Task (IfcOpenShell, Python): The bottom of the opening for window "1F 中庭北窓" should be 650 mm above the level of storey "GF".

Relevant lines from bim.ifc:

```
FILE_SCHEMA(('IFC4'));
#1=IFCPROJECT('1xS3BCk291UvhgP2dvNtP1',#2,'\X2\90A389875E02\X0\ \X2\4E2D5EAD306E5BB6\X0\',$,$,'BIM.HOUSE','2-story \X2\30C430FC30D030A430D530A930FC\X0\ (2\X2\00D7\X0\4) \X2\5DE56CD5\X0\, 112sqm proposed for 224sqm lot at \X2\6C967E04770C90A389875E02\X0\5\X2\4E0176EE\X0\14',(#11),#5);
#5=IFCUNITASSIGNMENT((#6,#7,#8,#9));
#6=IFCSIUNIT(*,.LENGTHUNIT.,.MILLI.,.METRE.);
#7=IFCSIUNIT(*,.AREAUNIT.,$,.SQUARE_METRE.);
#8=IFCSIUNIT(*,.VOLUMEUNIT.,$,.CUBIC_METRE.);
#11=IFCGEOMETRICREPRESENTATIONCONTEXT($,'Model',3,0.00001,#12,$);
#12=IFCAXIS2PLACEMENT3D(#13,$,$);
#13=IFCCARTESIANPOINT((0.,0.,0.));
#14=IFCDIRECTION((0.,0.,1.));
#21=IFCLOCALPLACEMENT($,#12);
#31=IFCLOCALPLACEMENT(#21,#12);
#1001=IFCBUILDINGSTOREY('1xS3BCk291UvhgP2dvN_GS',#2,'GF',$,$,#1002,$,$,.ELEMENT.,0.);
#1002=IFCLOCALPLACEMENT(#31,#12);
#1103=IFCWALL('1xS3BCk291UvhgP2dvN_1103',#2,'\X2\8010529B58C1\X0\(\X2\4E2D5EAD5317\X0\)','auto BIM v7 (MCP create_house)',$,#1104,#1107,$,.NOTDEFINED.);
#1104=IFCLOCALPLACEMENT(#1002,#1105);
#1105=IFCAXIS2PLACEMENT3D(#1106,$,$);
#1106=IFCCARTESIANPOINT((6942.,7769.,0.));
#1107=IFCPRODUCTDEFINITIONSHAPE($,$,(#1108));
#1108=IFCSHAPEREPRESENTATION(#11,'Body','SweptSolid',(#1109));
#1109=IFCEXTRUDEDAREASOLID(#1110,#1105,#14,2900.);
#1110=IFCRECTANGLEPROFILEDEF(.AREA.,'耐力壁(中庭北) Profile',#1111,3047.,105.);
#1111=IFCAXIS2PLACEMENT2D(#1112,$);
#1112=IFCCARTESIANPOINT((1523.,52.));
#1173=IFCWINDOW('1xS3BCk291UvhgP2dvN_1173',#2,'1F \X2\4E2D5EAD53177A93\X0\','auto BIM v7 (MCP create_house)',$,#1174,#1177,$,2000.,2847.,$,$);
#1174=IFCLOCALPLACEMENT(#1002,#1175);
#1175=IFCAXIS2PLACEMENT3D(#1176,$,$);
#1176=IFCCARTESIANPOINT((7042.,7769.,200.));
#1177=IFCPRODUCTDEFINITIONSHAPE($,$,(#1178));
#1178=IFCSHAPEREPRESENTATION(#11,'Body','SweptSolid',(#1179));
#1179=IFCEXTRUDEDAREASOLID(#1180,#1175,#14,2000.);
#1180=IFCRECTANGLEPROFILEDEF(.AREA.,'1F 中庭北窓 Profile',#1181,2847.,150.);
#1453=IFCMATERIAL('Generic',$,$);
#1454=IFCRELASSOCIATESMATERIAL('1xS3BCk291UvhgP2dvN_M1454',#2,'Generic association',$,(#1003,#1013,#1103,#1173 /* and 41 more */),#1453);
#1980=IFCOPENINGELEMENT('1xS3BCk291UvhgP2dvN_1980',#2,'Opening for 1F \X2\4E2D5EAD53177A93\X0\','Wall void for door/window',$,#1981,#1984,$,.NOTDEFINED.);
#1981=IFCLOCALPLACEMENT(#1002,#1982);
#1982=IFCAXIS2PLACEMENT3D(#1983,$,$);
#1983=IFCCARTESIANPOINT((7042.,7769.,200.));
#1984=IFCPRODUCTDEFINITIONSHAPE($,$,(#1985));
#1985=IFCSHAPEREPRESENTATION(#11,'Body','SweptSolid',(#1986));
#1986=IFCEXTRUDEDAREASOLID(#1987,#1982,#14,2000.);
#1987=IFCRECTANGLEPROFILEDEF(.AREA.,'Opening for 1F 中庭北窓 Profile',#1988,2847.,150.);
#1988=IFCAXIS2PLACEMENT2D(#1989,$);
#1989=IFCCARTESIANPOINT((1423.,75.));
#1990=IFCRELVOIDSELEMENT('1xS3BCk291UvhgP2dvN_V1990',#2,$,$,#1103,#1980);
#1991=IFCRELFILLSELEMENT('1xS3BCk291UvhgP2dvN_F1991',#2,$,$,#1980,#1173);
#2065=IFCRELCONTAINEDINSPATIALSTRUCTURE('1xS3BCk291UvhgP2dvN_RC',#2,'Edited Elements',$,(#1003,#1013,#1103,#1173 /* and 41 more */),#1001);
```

```python
import numpy as np
import ifcopenshell
import ifcopenshell.api.geometry
import ifcopenshell.geom
import ifcopenshell.util.element
import ifcopenshell.util.placement
import ifcopenshell.util.shape
import ifcopenshell.util.unit

model = ifcopenshell.open("bim.ifc")
unit_scale = ifcopenshell.util.unit.calculate_unit_scale(model)

window = model.by_guid("1xS3BCk291UvhgP2dvN_1173")
opening = window.FillsVoids[0].RelatingOpeningElement
storey = ifcopenshell.util.element.get_container(window, ifc_class="IfcBuildingStorey")
level = ifcopenshell.util.placement.get_local_placement(storey.ObjectPlacement)[2, 3]

# The opening's origin need not be at the sill, so measure its lowest point.
shape = ifcopenshell.geom.create_shape(ifcopenshell.geom.settings(), opening)
bottom = ifcopenshell.util.shape.get_shape_bottom_elevation(shape, shape.geometry) / unit_scale
dz = level + 0.65 / unit_scale - bottom

shift = np.array([0.0, 0.0, dz])
# The window is not placed relative to its opening, so move both.
for product in (opening, window):
    matrix = ifcopenshell.util.placement.get_local_placement(product.ObjectPlacement)
    matrix[:3, 3] += shift
    ifcopenshell.api.geometry.edit_object_placement(model, product=product, matrix=matrix, is_si=False)

print(f"moved by {dz * unit_scale:+.3f} m")

model.write("bim_edited.ifc")
```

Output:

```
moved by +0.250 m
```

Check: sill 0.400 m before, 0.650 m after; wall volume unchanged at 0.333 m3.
